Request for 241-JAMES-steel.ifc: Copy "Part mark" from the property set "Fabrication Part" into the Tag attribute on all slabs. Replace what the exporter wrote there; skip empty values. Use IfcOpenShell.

First a look at what the model holds.

```python
import ifcopenshell
import ifcopenshell.util.element

model = ifcopenshell.open("241-JAMES-steel.ifc")
print(model.schema)
slabs = model.by_type("IfcSlab")
print(len(slabs), "slabs")
for e in slabs[:8]:
    source = ifcopenshell.util.element.get_pset(e, "Fabrication Part", "Part mark")
    target = e.Tag
    print(e.id(), repr(source), repr(target), sep=" | ")
```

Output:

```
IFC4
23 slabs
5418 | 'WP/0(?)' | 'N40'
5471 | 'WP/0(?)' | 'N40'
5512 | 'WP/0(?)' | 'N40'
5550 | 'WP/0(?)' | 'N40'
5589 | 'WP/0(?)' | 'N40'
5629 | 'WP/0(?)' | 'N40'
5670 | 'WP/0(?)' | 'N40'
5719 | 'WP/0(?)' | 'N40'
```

```python
import ifcopenshell
import ifcopenshell.util.element

model = ifcopenshell.open("241-JAMES-steel.ifc")

count = 0
for e in model.by_type("IfcSlab"):
    value = ifcopenshell.util.element.get_pset(e, "Fabrication Part", "Part mark")
    current = e.Tag
    if not value or not value.strip() or current == value:
        continue
    e.Tag = value
    count += 1

print(count, "slabs updated")

model.write("241-JAMES-steel_rev.ifc")
```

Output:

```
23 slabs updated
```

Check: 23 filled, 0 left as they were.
